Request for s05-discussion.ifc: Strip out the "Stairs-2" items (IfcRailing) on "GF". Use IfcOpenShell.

First a look at what the model holds.

```python
import ifcopenshell
import ifcopenshell.util.element

model = ifcopenshell.open("s05-discussion.ifc")
print(model.schema)
storey = next(s for s in model.by_type("IfcBuildingStorey") if s.Name == "GF")
railings = [e for e in ifcopenshell.util.element.get_decomposition(storey) if e.is_a("IfcRailing")]
seen = {}
for e in railings:
    element_type = ifcopenshell.util.element.get_type(e)
    name = element_type.Name if element_type not in (None, e) else None
    seen[name] = seen.get(name, 0) + 1
for name, count in sorted(seen.items(), key=str):
    print(count, "x", name)
```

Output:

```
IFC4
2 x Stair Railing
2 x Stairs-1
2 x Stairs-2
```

```python
import ifcopenshell
import ifcopenshell.api.root
import ifcopenshell.util.element

model = ifcopenshell.open("s05-discussion.ifc")

storey = next(s for s in model.by_type("IfcBuildingStorey") if s.Name == "GF")
railings = [e for e in ifcopenshell.util.element.get_decomposition(storey) if e.is_a("IfcRailing")]
targets = [e for e in railings if (t := ifcopenshell.util.element.get_type(e)) not in (None, e) and t.Name == "Stairs-2"]

for e in targets:
    ifcopenshell.api.root.remove_product(model, product=e)
print(len(targets), "removed")

model.write("s05-discussion_updated.ifc")
```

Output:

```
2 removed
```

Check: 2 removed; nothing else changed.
